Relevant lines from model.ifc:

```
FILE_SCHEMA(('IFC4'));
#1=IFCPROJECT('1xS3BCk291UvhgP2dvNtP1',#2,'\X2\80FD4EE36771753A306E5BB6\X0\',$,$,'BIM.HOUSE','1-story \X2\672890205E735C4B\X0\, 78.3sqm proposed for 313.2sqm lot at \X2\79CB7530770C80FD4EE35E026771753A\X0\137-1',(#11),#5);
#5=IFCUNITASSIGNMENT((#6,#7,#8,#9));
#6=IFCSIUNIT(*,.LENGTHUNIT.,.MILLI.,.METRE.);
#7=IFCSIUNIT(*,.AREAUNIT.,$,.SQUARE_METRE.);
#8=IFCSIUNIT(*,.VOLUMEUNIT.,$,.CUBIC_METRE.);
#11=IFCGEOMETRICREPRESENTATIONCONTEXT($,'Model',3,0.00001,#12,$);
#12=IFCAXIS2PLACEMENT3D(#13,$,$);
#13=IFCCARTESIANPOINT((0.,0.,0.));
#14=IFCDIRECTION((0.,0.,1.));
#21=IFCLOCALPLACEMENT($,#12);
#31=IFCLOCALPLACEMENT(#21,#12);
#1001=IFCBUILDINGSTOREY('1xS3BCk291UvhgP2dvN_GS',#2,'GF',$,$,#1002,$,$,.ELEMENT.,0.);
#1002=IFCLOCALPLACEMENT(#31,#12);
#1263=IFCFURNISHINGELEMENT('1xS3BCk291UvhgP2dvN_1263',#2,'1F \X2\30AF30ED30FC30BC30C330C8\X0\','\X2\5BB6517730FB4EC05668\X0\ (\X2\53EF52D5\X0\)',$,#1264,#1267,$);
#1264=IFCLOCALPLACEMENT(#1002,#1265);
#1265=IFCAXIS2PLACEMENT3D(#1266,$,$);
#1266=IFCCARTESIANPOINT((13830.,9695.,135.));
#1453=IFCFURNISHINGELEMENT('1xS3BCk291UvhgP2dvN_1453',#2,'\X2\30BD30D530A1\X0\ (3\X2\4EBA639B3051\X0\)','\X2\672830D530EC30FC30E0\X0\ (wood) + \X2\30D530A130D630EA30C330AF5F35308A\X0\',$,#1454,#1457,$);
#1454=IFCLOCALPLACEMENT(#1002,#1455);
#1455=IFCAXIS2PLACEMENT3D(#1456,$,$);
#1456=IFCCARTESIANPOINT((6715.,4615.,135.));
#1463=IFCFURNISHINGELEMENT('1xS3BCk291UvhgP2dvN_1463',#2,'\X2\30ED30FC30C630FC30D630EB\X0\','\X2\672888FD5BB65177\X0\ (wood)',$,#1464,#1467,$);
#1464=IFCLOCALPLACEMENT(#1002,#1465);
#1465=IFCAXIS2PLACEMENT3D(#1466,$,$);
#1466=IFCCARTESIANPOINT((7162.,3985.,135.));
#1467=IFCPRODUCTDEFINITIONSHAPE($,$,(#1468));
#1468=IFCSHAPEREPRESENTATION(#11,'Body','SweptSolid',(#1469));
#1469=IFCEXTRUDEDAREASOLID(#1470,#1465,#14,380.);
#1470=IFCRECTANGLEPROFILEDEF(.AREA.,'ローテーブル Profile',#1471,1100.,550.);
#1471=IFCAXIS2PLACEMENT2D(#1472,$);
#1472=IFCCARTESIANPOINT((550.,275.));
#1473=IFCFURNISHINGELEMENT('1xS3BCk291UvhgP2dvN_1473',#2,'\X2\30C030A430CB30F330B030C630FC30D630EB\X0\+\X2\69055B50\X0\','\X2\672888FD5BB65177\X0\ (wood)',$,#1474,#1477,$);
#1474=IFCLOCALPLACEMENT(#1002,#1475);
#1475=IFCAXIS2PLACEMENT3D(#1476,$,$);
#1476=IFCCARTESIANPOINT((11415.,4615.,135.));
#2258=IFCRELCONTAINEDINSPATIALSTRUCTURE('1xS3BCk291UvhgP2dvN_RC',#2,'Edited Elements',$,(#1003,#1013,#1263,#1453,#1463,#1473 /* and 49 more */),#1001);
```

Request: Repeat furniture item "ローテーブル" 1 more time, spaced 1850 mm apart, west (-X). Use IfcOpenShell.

```python
import numpy as np
import ifcopenshell
import ifcopenshell.api.geometry
import ifcopenshell.api.root
import ifcopenshell.util.element
import ifcopenshell.util.placement

model = ifcopenshell.open("model.ifc")


def reuse_history(source, copy):
    """copy_class also copies each property set's owner history, people and application; keep the originals."""
    for rel in copy.IsDefinedBy:
        if rel.is_a("IfcRelDefinesByProperties") and (history := rel.RelatingPropertyDefinition.OwnerHistory):
            rel.RelatingPropertyDefinition.OwnerHistory = source.OwnerHistory
            ifcopenshell.util.element.remove_deep2(model, history)


source = model.by_guid("1xS3BCk291UvhgP2dvN_1463")
base = ifcopenshell.util.placement.get_local_placement(source.ObjectPlacement)
step = np.array([-1.0, 0.0, 0.0]) * 1850.0

for i in range(1, 2):
    copy = ifcopenshell.api.root.copy_class(model, product=source)
    copy.Representation = ifcopenshell.util.element.copy_deep(
        model, source.Representation, exclude=["IfcGeometricRepresentationContext", "IfcRepresentationMap"]
    )
    reuse_history(source, copy)
    matrix = base.copy()
    matrix[:3, 3] += i * step
    print("added at", matrix[:3, 3].round(3) + 0.0)
    ifcopenshell.api.geometry.edit_object_placement(model, product=copy, matrix=matrix, is_si=False)

model.write("model_v2.ifc")
```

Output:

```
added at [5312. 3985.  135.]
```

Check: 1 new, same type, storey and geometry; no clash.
